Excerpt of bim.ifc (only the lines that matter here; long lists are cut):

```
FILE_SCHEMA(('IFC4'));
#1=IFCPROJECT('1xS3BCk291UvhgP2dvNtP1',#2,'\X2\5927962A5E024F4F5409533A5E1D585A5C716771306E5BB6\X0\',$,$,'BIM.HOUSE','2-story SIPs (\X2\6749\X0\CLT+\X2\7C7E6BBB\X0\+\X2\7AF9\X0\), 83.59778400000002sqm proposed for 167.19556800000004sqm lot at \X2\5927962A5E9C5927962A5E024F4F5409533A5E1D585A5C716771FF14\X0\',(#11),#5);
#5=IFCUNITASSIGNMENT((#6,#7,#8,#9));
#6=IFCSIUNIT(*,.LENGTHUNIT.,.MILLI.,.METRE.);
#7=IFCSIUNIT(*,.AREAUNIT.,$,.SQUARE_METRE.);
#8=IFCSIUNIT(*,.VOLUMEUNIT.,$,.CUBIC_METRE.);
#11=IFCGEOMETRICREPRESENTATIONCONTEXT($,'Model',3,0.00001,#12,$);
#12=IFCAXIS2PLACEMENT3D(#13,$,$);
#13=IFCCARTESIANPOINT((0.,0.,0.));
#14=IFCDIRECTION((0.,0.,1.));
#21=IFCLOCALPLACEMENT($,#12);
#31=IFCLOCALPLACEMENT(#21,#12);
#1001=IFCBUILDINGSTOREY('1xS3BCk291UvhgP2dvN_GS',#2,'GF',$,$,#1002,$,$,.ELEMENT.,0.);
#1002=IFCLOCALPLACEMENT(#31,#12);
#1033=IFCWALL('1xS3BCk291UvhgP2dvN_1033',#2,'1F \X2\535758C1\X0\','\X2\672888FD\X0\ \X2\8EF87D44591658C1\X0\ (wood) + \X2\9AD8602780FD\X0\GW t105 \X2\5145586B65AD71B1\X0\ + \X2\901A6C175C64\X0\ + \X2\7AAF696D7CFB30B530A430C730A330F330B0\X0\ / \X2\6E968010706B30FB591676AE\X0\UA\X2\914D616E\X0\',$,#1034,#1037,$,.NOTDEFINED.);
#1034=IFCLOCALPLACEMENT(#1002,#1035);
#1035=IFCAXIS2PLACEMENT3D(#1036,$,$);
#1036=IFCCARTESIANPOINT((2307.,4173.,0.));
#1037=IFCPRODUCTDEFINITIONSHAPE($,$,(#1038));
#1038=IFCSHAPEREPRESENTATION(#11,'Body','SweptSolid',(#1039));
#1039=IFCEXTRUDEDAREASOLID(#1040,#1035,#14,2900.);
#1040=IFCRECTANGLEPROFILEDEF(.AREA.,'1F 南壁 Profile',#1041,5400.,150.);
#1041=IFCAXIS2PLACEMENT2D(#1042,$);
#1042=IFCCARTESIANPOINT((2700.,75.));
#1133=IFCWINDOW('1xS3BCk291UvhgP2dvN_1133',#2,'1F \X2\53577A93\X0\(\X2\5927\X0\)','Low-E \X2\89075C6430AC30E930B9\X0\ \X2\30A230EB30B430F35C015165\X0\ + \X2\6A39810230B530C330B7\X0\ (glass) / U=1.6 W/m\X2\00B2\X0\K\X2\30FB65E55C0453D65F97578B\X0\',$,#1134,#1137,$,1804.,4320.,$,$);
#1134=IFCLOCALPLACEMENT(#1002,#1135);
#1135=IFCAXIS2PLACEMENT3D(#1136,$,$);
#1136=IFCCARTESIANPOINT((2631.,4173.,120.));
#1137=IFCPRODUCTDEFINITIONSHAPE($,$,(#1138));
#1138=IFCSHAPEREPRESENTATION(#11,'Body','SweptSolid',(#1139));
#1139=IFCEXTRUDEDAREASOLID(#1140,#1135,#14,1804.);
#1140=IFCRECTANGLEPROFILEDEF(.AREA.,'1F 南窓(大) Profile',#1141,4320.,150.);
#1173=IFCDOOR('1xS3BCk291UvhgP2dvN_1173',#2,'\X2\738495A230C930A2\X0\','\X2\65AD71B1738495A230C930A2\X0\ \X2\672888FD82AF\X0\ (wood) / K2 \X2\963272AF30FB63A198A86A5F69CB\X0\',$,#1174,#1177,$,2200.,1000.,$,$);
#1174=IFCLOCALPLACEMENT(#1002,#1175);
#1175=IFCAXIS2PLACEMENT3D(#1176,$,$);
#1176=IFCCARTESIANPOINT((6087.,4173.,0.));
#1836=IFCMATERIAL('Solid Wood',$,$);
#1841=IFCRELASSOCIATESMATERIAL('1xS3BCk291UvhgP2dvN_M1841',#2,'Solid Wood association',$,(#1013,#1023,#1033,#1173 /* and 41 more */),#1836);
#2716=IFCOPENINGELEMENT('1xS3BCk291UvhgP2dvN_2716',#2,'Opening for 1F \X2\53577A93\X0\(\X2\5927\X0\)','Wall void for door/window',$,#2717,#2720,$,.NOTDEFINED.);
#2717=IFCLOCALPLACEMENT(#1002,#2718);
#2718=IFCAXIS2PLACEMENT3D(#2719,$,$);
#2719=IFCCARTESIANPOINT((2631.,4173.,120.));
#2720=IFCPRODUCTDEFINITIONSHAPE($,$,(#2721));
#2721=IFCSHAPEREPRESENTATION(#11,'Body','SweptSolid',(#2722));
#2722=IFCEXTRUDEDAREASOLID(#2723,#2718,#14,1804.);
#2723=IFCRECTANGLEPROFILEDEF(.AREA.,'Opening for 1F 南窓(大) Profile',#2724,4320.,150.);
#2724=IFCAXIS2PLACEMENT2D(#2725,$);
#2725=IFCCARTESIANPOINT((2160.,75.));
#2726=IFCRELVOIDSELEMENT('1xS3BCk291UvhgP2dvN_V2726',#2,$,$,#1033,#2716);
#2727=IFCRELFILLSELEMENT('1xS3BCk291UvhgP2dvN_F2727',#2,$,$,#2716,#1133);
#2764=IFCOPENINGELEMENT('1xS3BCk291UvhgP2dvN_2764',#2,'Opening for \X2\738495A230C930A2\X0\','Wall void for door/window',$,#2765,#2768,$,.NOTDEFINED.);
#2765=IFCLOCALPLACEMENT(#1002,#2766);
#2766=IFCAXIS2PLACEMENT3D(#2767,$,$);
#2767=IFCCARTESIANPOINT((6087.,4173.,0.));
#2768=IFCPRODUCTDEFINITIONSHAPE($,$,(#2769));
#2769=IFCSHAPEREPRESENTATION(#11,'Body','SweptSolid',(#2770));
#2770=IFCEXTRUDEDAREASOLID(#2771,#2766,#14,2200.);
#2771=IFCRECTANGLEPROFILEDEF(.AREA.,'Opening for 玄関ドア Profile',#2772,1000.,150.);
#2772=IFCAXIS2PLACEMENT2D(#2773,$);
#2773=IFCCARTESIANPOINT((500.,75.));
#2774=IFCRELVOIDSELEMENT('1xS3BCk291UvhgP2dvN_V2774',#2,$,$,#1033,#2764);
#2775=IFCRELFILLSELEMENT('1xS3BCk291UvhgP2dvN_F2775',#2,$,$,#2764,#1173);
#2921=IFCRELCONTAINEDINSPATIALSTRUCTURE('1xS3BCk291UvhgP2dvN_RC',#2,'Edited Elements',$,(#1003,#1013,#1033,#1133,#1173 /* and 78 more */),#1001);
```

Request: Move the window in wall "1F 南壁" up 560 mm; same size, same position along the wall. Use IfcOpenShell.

```python
import numpy as np
import ifcopenshell
import ifcopenshell.api.geometry
import ifcopenshell.util.placement
import ifcopenshell.util.unit

model = ifcopenshell.open("bim.ifc")
unit_scale = ifcopenshell.util.unit.calculate_unit_scale(model)

window = model.by_guid("1xS3BCk291UvhgP2dvN_1133")
opening = window.FillsVoids[0].RelatingOpeningElement
dz = 0.56 / unit_scale

shift = np.array([0.0, 0.0, dz])
# The window is not placed relative to its opening, so move both.
for product in (opening, window):
    matrix = ifcopenshell.util.placement.get_local_placement(product.ObjectPlacement)
    matrix[:3, 3] += shift
    ifcopenshell.api.geometry.edit_object_placement(model, product=product, matrix=matrix, is_si=False)

print(f"moved by {dz * unit_scale:+.3f} m")

model.write("bim_rev.ifc")
```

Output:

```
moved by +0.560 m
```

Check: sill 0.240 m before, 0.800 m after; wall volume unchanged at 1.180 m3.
